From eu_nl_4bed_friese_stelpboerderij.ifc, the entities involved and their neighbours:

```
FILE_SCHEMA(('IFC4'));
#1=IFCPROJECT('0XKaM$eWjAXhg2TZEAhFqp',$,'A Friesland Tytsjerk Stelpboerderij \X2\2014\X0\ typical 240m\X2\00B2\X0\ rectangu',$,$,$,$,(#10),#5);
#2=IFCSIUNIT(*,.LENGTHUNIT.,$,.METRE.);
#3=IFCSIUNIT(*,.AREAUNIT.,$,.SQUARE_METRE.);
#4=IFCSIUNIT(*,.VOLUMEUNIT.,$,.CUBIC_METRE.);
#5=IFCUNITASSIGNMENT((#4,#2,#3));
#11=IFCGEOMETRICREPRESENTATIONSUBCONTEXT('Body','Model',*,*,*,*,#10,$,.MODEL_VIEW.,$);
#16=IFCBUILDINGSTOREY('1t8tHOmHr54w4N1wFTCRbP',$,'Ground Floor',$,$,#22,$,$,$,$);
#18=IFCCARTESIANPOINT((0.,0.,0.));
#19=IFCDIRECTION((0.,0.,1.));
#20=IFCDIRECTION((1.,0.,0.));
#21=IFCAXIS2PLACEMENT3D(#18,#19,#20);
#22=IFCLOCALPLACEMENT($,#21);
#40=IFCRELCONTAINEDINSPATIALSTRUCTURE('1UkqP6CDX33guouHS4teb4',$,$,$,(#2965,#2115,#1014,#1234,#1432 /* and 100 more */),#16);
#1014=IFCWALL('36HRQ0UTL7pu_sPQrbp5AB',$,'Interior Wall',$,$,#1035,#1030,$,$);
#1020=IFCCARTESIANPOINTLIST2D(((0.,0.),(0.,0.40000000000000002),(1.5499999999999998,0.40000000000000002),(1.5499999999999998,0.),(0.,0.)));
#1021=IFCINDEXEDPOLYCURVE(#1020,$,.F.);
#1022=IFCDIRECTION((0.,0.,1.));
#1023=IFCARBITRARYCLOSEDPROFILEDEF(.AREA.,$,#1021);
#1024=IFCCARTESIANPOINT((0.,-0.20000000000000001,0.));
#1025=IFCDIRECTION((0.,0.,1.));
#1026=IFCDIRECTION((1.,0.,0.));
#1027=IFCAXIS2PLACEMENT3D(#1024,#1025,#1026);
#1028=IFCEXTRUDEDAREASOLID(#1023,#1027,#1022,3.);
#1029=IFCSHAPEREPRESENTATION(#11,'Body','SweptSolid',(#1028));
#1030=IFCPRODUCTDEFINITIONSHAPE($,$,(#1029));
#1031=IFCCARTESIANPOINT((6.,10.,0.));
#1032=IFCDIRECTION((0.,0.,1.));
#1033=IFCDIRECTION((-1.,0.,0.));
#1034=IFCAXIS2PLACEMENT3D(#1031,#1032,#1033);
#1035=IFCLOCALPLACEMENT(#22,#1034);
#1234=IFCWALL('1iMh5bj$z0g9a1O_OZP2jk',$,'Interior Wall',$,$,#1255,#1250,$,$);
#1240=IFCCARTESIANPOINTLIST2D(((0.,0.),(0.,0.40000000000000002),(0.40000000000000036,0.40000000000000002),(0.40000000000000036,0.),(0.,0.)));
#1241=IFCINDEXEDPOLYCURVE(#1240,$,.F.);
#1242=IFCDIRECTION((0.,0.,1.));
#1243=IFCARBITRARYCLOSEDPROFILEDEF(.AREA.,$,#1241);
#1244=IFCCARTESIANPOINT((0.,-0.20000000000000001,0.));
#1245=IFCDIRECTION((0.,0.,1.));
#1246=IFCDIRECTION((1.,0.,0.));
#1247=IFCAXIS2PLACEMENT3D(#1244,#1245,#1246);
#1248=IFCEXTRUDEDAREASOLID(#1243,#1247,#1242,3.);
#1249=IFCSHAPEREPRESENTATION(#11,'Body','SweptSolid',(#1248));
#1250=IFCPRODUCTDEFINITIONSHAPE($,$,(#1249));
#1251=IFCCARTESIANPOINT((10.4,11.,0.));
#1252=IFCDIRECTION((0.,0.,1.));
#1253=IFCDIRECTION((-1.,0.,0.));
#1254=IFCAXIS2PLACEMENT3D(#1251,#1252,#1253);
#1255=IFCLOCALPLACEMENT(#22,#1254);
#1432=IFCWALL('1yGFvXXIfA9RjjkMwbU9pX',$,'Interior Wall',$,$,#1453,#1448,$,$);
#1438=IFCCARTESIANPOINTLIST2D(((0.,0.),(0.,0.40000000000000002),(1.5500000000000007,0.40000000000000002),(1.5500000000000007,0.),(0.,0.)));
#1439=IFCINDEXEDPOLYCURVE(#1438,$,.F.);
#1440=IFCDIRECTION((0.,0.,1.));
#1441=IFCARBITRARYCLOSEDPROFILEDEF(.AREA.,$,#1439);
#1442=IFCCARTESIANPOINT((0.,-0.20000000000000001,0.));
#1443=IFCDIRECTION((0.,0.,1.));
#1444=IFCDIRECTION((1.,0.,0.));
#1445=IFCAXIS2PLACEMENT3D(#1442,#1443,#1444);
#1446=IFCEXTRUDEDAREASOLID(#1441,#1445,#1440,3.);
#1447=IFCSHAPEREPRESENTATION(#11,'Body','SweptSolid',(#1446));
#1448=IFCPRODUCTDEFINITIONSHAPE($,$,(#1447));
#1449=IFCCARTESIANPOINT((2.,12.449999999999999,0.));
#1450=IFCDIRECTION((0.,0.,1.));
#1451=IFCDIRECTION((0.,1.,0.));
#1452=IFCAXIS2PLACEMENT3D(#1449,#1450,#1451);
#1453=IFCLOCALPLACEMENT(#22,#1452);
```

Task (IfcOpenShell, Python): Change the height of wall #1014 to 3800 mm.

```python
import ifcopenshell
import ifcopenshell.geom
import ifcopenshell.util.representation
import ifcopenshell.util.shape
import ifcopenshell.util.unit

model = ifcopenshell.open("eu_nl_4bed_friese_stelpboerderij.ifc")
unit_scale = ifcopenshell.util.unit.calculate_unit_scale(model)
settings = ifcopenshell.geom.settings()


def volume(element):
    """Net volume in cubic metres, openings subtracted."""
    shape = ifcopenshell.geom.create_shape(settings, element)
    return ifcopenshell.util.shape.get_volume(shape.geometry)


wall = model.by_guid("36HRQ0UTL7pu_sPQrbp5AB")
before = volume(wall)

body = ifcopenshell.util.representation.get_representation(wall, "Model", "Body")
solid = body.Items[0]
old_height = solid.Depth
solid.Depth = 3.8 / unit_scale
after = volume(wall)

print(f"height {old_height:g} -> {solid.Depth:g}, volume {before:.3f} -> {after:.3f} m3")

model.write("eu_nl_4bed_friese_stelpboerderij_updated.ifc")
```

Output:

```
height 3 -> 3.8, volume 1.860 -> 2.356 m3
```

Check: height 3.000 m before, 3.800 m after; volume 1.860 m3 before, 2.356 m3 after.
